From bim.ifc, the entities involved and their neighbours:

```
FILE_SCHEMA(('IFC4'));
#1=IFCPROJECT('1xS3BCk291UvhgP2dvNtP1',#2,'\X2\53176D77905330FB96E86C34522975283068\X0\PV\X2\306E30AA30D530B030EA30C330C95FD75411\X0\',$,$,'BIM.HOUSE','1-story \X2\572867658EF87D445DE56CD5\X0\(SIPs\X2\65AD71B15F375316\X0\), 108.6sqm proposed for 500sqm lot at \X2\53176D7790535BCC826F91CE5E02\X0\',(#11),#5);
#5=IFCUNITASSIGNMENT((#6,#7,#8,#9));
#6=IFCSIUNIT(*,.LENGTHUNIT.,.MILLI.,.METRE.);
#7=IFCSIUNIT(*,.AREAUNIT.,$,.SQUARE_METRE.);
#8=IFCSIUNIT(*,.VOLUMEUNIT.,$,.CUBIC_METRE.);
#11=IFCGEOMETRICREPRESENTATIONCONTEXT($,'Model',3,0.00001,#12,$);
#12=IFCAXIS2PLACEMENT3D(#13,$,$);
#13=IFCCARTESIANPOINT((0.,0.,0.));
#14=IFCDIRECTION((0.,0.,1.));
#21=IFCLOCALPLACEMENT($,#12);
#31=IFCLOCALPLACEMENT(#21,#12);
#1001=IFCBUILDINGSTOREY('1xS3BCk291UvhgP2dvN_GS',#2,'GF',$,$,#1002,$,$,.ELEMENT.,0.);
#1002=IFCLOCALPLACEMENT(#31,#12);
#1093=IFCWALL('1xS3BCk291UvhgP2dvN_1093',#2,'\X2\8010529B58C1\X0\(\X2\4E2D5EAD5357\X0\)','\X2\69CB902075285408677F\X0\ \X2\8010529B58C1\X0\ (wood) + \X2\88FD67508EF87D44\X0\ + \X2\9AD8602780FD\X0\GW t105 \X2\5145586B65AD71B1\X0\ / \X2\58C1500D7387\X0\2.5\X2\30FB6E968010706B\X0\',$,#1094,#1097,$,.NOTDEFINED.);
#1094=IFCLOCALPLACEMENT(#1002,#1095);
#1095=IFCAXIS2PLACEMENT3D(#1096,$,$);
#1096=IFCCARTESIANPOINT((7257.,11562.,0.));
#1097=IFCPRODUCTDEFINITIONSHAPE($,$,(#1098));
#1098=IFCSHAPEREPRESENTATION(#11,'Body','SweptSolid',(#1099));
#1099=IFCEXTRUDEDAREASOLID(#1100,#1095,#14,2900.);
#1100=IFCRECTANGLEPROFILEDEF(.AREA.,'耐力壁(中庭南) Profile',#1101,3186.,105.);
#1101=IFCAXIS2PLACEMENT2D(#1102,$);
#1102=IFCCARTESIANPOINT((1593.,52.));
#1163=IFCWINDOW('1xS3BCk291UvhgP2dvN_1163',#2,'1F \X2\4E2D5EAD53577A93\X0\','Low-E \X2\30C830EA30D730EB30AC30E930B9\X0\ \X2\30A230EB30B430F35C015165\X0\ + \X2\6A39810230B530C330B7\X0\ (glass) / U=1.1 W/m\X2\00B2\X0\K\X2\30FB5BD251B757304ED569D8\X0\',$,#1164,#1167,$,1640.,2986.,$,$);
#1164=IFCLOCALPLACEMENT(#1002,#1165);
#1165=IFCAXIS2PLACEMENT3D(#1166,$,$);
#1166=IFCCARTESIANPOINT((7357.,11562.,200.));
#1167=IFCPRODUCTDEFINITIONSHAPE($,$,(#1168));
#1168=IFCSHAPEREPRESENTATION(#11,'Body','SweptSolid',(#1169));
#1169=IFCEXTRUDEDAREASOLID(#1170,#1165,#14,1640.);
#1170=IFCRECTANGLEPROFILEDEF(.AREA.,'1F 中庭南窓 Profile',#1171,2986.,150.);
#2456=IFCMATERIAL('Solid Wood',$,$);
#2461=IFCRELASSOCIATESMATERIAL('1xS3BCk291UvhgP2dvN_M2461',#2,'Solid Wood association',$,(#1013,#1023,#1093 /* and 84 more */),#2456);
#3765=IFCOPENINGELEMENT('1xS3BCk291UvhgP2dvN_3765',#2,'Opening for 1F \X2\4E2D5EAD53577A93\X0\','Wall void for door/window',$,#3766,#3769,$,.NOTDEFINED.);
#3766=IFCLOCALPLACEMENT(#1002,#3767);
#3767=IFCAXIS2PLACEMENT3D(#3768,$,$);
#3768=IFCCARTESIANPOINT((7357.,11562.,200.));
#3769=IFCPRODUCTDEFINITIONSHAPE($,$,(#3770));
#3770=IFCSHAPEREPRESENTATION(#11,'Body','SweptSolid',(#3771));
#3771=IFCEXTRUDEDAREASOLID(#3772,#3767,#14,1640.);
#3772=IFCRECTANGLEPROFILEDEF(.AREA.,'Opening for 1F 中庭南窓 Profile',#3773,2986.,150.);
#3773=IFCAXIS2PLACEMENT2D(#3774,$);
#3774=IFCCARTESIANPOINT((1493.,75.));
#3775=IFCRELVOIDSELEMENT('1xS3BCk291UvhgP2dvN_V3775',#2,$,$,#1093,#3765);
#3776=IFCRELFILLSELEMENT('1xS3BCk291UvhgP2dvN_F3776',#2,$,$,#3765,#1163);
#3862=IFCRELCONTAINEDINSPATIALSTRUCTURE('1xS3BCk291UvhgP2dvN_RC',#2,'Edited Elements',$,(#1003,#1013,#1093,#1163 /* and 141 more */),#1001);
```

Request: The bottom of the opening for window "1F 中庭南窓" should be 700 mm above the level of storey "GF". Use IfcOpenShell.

```python
import numpy as np
import ifcopenshell
import ifcopenshell.api.geometry
import ifcopenshell.geom
import ifcopenshell.util.element
import ifcopenshell.util.placement
import ifcopenshell.util.shape
import ifcopenshell.util.unit

model = ifcopenshell.open("bim.ifc")
unit_scale = ifcopenshell.util.unit.calculate_unit_scale(model)

window = model.by_id(1163)
opening = window.FillsVoids[0].RelatingOpeningElement
storey = ifcopenshell.util.element.get_container(window, ifc_class="IfcBuildingStorey")
level = ifcopenshell.util.placement.get_local_placement(storey.ObjectPlacement)[2, 3]

# The opening's origin need not be at the sill, so measure its lowest point.
shape = ifcopenshell.geom.create_shape(ifcopenshell.geom.settings(), opening)
bottom = ifcopenshell.util.shape.get_shape_bottom_elevation(shape, shape.geometry) / unit_scale
dz = level + 0.7 / unit_scale - bottom

shift = np.array([0.0, 0.0, dz])
# The window is not placed relative to its opening, so move both.
for product in (opening, window):
    matrix = ifcopenshell.util.placement.get_local_placement(product.ObjectPlacement)
    matrix[:3, 3] += shift
    ifcopenshell.api.geometry.edit_object_placement(model, product=product, matrix=matrix, is_si=False)

print(f"moved by {dz * unit_scale:+.3f} m")

model.write("bim-out.ifc")
```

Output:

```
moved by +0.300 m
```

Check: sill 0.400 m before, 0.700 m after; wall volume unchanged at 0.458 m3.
